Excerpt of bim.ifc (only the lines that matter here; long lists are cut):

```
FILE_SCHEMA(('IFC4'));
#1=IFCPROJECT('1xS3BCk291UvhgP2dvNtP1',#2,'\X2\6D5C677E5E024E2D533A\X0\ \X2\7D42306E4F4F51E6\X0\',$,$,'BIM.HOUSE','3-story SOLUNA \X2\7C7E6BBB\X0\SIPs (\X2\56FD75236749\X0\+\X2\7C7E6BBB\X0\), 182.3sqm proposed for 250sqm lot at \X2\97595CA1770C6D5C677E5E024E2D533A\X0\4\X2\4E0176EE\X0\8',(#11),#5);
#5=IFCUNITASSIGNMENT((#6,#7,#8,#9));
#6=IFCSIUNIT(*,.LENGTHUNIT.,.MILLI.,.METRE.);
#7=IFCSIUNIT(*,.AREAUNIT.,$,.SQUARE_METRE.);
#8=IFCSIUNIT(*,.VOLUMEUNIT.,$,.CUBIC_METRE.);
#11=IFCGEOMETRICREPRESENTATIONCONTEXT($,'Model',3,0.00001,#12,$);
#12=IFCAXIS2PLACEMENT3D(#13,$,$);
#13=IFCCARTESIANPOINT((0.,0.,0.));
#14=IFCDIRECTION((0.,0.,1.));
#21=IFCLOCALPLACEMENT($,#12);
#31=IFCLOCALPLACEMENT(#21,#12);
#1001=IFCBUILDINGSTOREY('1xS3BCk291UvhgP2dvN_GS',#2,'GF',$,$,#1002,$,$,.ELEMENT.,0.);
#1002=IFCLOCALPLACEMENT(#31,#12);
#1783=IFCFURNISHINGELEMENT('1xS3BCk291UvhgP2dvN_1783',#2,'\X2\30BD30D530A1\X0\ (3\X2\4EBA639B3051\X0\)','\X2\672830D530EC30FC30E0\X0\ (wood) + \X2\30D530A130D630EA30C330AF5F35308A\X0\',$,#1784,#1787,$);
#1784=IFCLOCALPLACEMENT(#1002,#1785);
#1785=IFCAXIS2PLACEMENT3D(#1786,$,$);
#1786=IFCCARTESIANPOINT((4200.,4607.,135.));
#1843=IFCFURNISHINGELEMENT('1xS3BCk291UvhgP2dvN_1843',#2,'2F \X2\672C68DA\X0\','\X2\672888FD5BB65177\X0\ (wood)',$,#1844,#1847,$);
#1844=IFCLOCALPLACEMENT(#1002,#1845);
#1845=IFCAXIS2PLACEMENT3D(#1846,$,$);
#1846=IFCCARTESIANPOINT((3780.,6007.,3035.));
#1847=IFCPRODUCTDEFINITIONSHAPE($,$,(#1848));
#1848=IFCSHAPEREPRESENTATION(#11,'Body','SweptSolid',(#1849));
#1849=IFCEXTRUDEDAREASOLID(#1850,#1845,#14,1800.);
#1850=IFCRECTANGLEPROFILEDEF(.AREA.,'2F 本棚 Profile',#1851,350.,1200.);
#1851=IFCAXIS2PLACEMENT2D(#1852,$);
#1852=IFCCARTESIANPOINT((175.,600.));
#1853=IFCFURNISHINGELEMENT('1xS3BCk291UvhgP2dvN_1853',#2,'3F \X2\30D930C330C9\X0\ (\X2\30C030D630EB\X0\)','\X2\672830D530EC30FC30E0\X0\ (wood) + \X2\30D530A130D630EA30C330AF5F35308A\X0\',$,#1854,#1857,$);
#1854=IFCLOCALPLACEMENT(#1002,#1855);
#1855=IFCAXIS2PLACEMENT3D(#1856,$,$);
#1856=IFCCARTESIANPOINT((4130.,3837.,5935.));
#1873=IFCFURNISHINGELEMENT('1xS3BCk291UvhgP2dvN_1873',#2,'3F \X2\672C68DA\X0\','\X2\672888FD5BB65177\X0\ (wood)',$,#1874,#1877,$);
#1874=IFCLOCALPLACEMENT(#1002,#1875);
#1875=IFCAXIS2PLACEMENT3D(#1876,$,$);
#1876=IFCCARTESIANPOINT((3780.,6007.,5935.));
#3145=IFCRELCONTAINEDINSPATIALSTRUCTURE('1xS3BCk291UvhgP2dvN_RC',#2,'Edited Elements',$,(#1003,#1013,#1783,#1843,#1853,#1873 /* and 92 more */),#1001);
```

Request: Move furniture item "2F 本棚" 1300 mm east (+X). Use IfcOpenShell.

```python
import ifcopenshell
import ifcopenshell.api.geometry
import ifcopenshell.util.placement
import ifcopenshell.util.unit

model = ifcopenshell.open("bim.ifc")
unit_scale = ifcopenshell.util.unit.calculate_unit_scale(model)

item = model.by_guid("1xS3BCk291UvhgP2dvN_1843")
matrix = ifcopenshell.util.placement.get_local_placement(item.ObjectPlacement)
matrix[0, 3] += 1.3 / unit_scale
ifcopenshell.api.geometry.edit_object_placement(model, product=item, matrix=matrix, is_si=False)

print(ifcopenshell.util.placement.get_local_placement(item.ObjectPlacement).round(3) + 0.0)

model.write("bim_updated.ifc")
```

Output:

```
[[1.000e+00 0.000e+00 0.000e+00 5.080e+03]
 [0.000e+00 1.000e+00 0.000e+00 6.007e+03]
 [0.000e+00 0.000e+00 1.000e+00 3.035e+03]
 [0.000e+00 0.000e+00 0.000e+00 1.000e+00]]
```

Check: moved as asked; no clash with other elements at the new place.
